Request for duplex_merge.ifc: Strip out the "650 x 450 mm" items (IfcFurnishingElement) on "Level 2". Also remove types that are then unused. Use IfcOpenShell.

First a look at what the model holds.

```python
import ifcopenshell
import ifcopenshell.util.element

model = ifcopenshell.open("duplex_merge.ifc")
print(model.schema)
storey = next(s for s in model.by_type("IfcBuildingStorey") if s.Name == "Level 2")
furniture = [e for e in ifcopenshell.util.element.get_decomposition(storey) if e.is_a("IfcFurnishingElement")]
seen = {}
for e in furniture:
    element_type = ifcopenshell.util.element.get_type(e)
    name = element_type.Name if element_type not in (None, e) else None
    seen[name] = seen.get(name, 0) + 1
for name, count in sorted(seen.items(), key=str):
    print(count, "x", name)
```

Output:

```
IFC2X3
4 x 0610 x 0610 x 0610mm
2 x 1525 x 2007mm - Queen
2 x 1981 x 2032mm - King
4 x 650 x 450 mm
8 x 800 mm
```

```python
import ifcopenshell
import ifcopenshell.api.root
import ifcopenshell.util.element

model = ifcopenshell.open("duplex_merge.ifc")

storey = next(s for s in model.by_type("IfcBuildingStorey") if s.Name == "Level 2")
furniture = [e for e in ifcopenshell.util.element.get_decomposition(storey) if e.is_a("IfcFurnishingElement")]
targets = [e for e in furniture if (t := ifcopenshell.util.element.get_type(e)) not in (None, e) and t.Name == "650 x 450 mm"]
types = {ifcopenshell.util.element.get_type(e) for e in targets} - {None, *targets}

for e in targets:
    ifcopenshell.api.root.remove_product(model, product=e)
print(len(targets), "removed")

unused = [t for t in types if not ifcopenshell.util.element.get_types(t)]
for t in unused:
    ifcopenshell.api.root.remove_product(model, product=t)
print(len(unused), "unused types removed")

model.write("duplex_merge_v2.ifc")
```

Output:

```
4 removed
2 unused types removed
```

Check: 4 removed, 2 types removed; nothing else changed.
